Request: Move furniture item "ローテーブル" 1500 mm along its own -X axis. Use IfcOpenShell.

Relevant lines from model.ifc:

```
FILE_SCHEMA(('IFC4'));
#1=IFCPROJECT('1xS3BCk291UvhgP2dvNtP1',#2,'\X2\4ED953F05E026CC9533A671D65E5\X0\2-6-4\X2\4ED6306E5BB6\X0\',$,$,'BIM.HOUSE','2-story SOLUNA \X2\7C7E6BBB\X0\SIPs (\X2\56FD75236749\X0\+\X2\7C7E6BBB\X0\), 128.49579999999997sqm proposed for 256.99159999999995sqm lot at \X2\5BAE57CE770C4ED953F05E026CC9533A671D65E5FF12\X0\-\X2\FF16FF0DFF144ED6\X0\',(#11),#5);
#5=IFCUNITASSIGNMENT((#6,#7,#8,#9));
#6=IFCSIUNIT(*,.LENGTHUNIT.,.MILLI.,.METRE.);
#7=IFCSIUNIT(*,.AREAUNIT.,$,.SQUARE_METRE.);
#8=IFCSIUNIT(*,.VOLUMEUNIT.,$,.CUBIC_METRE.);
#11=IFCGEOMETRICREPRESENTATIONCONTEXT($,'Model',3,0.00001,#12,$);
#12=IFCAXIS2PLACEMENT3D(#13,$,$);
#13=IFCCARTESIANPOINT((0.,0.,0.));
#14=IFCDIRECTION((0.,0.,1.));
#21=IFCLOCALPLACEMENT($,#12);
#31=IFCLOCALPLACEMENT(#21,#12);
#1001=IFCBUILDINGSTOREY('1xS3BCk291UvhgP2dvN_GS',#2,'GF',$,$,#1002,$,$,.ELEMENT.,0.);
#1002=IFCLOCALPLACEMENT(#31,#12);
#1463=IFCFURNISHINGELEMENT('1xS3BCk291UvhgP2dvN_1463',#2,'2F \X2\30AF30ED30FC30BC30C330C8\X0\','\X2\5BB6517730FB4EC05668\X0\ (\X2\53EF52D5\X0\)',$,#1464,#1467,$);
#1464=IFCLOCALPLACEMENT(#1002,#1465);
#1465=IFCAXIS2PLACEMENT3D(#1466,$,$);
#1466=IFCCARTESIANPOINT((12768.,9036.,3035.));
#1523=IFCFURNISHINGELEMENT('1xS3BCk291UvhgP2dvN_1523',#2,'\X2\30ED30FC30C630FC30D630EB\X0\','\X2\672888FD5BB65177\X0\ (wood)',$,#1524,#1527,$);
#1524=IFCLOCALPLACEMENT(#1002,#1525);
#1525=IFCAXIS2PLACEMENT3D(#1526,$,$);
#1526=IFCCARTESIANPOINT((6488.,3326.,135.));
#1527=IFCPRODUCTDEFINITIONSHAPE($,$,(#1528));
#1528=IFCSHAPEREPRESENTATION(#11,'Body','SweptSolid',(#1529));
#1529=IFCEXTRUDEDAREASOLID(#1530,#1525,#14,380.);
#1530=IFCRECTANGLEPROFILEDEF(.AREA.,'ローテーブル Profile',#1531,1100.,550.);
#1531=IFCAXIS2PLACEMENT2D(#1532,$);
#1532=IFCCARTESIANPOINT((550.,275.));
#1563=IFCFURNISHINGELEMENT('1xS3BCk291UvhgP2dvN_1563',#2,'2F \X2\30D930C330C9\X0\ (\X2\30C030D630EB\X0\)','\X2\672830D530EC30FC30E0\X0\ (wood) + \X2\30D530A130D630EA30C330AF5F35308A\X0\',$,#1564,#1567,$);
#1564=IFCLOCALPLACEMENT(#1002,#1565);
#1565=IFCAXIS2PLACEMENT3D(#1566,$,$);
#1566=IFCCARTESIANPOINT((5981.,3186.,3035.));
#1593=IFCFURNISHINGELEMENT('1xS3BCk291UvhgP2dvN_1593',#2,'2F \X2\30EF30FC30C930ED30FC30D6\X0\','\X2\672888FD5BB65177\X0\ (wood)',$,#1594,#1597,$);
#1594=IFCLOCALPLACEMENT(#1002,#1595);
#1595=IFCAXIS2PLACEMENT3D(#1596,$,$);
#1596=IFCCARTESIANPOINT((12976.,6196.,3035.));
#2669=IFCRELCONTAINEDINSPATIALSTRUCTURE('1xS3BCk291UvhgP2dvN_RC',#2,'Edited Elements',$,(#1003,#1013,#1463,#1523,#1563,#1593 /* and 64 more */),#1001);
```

```python
import ifcopenshell
import ifcopenshell.api.geometry
import ifcopenshell.util.placement
import ifcopenshell.util.unit

model = ifcopenshell.open("model.ifc")
unit_scale = ifcopenshell.util.unit.calculate_unit_scale(model)

item = model.by_id(1523)
matrix = ifcopenshell.util.placement.get_local_placement(item.ObjectPlacement)
matrix[:3, 3] -= matrix[:3, 0] * 1.5 / unit_scale
ifcopenshell.api.geometry.edit_object_placement(model, product=item, matrix=matrix, is_si=False)

print(ifcopenshell.util.placement.get_local_placement(item.ObjectPlacement).round(3) + 0.0)

model.write("model_v2.ifc")
```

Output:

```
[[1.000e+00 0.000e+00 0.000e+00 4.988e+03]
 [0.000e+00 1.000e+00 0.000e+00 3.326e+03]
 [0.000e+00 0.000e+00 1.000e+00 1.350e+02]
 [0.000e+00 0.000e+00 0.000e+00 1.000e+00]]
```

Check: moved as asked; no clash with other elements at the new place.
